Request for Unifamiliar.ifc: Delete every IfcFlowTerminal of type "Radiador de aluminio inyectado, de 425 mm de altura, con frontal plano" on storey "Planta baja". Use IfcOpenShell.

First a look at what the model holds.

```python
import ifcopenshell
import ifcopenshell.util.element

model = ifcopenshell.open("Unifamiliar.ifc")
print(model.schema)
storey = next(s for s in model.by_type("IfcBuildingStorey") if s.Name == "Planta baja")
terminals = [e for e in ifcopenshell.util.element.get_decomposition(storey) if e.is_a("IfcFlowTerminal")]
seen = {}
for e in terminals:
    element_type = ifcopenshell.util.element.get_type(e)
    name = element_type.Name if element_type not in (None, e) else None
    seen[name] = seen.get(name, 0) + 1
for name, count in sorted(seen.items(), key=str):
    print(count, "x", name)
```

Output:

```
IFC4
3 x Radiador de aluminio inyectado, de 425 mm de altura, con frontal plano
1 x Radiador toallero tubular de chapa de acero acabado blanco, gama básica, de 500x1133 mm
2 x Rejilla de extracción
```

```python
import ifcopenshell
import ifcopenshell.api.root
import ifcopenshell.util.element

model = ifcopenshell.open("Unifamiliar.ifc")

storey = next(s for s in model.by_type("IfcBuildingStorey") if s.Name == "Planta baja")
terminals = [e for e in ifcopenshell.util.element.get_decomposition(storey) if e.is_a("IfcFlowTerminal")]
targets = [e for e in terminals if (t := ifcopenshell.util.element.get_type(e)) not in (None, e) and t.Name == "Radiador de aluminio inyectado, de 425 mm de altura, con frontal plano"]

for e in targets:
    ifcopenshell.api.root.remove_product(model, product=e)
print(len(targets), "removed")

model.write("Unifamiliar_v2.ifc")
```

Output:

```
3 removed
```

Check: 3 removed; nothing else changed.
